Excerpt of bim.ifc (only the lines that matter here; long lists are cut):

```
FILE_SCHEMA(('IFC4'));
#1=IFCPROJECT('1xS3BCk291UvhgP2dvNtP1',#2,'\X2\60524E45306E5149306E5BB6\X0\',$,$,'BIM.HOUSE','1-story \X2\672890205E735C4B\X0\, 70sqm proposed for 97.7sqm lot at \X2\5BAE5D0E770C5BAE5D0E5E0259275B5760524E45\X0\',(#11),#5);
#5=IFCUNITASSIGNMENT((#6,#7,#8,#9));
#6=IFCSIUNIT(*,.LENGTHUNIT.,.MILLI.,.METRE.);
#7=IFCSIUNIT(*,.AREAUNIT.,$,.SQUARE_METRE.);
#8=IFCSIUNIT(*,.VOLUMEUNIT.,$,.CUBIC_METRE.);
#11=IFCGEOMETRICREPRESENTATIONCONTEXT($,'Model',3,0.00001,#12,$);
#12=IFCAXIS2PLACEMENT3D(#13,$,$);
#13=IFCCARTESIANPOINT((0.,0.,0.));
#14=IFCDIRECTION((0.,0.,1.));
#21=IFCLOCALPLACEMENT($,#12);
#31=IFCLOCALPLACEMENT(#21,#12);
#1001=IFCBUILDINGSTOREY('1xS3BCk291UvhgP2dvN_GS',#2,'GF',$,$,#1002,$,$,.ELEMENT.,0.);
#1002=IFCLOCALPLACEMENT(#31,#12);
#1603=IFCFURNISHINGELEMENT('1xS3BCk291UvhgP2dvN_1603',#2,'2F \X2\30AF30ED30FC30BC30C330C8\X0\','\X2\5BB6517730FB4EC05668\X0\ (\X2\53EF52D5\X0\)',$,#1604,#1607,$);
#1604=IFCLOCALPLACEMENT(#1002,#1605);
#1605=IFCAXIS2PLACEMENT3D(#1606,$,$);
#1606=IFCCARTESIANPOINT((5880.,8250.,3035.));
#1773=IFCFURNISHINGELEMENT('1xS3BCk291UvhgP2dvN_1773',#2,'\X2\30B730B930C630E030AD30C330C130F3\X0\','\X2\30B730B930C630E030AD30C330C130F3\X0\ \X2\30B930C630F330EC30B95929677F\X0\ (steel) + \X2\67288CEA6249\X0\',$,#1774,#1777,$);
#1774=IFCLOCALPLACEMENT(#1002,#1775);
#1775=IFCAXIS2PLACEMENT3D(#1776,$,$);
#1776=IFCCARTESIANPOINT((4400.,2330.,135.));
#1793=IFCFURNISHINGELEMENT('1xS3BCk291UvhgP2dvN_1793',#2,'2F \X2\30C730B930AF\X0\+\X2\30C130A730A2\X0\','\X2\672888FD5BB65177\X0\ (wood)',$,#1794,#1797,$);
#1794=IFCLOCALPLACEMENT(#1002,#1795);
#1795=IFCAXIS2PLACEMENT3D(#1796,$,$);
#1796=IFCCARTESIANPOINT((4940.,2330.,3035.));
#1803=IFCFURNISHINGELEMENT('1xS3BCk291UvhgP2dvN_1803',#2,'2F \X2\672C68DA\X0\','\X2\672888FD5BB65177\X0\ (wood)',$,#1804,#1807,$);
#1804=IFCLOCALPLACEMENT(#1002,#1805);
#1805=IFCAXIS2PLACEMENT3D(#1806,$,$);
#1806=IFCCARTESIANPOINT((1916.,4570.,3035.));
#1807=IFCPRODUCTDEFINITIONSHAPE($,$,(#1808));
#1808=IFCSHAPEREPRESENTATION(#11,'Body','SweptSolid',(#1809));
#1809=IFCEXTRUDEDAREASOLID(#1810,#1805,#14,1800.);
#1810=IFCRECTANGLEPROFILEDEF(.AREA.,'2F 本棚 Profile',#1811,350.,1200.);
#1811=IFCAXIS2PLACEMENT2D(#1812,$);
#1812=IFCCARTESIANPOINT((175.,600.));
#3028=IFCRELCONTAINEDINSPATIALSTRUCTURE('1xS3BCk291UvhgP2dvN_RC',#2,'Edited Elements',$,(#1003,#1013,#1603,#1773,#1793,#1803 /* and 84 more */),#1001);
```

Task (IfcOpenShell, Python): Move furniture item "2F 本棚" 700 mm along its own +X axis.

```python
import ifcopenshell
import ifcopenshell.api.geometry
import ifcopenshell.util.placement

model = ifcopenshell.open("bim.ifc")

item = model.by_guid("1xS3BCk291UvhgP2dvN_1803")
matrix = ifcopenshell.util.placement.get_local_placement(item.ObjectPlacement)
matrix[:3, 3] += matrix[:3, 0] * 700.0
ifcopenshell.api.geometry.edit_object_placement(model, product=item, matrix=matrix, is_si=False)

print(ifcopenshell.util.placement.get_local_placement(item.ObjectPlacement).round(3) + 0.0)

model.write("bim_edited.ifc")
```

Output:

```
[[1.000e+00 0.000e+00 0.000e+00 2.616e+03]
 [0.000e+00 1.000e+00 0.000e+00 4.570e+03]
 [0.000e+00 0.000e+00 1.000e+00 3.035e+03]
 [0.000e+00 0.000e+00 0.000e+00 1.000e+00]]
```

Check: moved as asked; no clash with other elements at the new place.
